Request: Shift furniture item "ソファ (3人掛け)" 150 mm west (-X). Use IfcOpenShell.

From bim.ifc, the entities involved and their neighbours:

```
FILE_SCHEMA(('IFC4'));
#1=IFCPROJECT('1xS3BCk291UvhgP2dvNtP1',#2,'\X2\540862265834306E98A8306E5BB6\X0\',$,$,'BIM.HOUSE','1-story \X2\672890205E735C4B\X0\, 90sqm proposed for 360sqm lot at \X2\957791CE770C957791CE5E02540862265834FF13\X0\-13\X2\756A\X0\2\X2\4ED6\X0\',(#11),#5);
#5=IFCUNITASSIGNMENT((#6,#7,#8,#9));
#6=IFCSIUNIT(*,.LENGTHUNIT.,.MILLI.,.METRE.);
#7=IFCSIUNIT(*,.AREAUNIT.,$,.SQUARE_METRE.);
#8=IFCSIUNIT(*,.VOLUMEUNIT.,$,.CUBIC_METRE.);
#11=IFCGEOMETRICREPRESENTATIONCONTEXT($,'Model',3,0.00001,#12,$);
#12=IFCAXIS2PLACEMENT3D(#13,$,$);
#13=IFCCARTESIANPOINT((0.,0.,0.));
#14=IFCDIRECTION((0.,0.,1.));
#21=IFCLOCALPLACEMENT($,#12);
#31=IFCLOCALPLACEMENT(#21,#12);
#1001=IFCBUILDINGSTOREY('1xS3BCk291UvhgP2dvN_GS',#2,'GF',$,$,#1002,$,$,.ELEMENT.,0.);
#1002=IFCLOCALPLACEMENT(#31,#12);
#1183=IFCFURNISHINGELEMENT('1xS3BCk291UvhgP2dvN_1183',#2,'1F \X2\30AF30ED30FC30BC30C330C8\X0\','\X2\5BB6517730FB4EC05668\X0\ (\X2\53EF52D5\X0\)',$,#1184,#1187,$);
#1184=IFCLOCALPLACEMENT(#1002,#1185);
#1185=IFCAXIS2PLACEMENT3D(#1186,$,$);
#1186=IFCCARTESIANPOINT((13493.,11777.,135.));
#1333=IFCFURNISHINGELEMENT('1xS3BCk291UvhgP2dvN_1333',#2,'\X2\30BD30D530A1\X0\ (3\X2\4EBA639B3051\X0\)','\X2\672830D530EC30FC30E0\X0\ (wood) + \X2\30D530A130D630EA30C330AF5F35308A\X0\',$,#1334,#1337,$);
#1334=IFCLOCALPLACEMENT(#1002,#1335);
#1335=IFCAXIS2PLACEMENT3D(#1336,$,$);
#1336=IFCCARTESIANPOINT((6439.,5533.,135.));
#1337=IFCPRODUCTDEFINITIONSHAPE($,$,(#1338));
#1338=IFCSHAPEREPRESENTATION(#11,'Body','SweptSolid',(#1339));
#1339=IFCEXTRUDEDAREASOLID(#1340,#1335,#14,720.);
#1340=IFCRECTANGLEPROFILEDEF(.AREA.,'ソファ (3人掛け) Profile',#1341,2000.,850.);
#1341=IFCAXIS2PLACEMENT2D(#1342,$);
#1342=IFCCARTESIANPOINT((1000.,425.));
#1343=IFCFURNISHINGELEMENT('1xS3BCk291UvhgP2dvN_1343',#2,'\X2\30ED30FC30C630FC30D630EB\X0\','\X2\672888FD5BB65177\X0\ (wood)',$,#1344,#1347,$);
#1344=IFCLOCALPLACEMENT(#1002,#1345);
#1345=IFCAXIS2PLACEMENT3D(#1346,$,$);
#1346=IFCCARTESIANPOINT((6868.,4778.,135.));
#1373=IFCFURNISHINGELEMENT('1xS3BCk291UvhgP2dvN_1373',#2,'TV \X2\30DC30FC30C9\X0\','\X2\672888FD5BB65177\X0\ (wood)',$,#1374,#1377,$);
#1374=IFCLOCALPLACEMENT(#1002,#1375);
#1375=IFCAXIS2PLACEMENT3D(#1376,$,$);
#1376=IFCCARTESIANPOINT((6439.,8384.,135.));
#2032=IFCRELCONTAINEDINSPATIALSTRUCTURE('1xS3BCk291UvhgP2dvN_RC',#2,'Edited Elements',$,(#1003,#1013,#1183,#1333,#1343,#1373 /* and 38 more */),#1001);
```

```python
import ifcopenshell
import ifcopenshell.api.geometry
import ifcopenshell.util.placement
import ifcopenshell.util.unit

model = ifcopenshell.open("bim.ifc")
unit_scale = ifcopenshell.util.unit.calculate_unit_scale(model)

item = model.by_id(1333)
matrix = ifcopenshell.util.placement.get_local_placement(item.ObjectPlacement)
matrix[0, 3] -= 0.15 / unit_scale
ifcopenshell.api.geometry.edit_object_placement(model, product=item, matrix=matrix, is_si=False)

print(ifcopenshell.util.placement.get_local_placement(item.ObjectPlacement).round(3) + 0.0)

model.write("bim-out.ifc")
```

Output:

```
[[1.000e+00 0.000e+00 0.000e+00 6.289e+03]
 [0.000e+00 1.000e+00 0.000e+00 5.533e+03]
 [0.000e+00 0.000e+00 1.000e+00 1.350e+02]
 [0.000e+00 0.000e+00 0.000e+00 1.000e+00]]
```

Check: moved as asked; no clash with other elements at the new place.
